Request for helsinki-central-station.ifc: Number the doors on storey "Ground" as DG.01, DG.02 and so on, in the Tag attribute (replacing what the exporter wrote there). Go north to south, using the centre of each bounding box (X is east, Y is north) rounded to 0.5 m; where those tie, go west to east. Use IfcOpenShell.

First a look at what the model holds.

```python
import ifcopenshell
import ifcopenshell.util.element
import ifcopenshell.util.placement

model = ifcopenshell.open("helsinki-central-station.ifc")
print(model.schema)
storey = next(s for s in model.by_type("IfcBuildingStorey") if s.Name == "Ground")
doors = [e for e in ifcopenshell.util.element.get_decomposition(storey) if e.is_a("IfcDoor")]
for e in sorted(doors, key=lambda e: e.id()):
    origin = ifcopenshell.util.placement.get_local_placement(e.ObjectPlacement)[:3, 3]
    print(e.id(), e.Tag, e.Name, origin.round(2) + 0.0, sep=" | ")
```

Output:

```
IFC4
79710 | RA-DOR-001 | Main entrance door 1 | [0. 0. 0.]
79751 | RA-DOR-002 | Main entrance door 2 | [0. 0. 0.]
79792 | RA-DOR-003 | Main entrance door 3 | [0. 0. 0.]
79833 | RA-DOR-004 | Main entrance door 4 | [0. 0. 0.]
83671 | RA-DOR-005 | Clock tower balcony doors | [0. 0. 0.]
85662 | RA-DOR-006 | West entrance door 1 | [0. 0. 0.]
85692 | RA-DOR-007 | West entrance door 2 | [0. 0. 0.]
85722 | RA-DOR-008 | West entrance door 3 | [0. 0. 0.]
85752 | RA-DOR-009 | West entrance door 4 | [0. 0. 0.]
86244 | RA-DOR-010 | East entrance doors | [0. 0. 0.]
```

```python
import ifcopenshell
import ifcopenshell.geom
import ifcopenshell.util.element
import ifcopenshell.util.shape

model = ifcopenshell.open("helsinki-central-station.ifc")
settings = ifcopenshell.geom.settings()
settings.set("use-world-coords", True)


def centre(element):
    shape = ifcopenshell.geom.create_shape(settings, element)
    return ifcopenshell.util.shape.get_bbox_centroid(shape.geometry)


storey = next(s for s in model.by_type("IfcBuildingStorey") if s.Name == "Ground")
doors = [e for e in ifcopenshell.util.element.get_decomposition(storey) if e.is_a("IfcDoor")]

# Insertion points can sit at a corner or the storey origin, so sort by the geometry (in metres).
centres = {e: centre(e) for e in doors}
doors.sort(key=lambda e: (-round(centres[e][1] / 0.5), centres[e][0]))

for i, e in enumerate(doors, start=1):
    number = f"DG.{i:02d}"
    e.Tag = number
    print(e.id(), number)

model.write("helsinki-central-station_rev.ifc")
```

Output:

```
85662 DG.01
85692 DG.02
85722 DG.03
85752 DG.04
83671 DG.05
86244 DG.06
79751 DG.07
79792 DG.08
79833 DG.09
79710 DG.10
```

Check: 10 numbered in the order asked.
